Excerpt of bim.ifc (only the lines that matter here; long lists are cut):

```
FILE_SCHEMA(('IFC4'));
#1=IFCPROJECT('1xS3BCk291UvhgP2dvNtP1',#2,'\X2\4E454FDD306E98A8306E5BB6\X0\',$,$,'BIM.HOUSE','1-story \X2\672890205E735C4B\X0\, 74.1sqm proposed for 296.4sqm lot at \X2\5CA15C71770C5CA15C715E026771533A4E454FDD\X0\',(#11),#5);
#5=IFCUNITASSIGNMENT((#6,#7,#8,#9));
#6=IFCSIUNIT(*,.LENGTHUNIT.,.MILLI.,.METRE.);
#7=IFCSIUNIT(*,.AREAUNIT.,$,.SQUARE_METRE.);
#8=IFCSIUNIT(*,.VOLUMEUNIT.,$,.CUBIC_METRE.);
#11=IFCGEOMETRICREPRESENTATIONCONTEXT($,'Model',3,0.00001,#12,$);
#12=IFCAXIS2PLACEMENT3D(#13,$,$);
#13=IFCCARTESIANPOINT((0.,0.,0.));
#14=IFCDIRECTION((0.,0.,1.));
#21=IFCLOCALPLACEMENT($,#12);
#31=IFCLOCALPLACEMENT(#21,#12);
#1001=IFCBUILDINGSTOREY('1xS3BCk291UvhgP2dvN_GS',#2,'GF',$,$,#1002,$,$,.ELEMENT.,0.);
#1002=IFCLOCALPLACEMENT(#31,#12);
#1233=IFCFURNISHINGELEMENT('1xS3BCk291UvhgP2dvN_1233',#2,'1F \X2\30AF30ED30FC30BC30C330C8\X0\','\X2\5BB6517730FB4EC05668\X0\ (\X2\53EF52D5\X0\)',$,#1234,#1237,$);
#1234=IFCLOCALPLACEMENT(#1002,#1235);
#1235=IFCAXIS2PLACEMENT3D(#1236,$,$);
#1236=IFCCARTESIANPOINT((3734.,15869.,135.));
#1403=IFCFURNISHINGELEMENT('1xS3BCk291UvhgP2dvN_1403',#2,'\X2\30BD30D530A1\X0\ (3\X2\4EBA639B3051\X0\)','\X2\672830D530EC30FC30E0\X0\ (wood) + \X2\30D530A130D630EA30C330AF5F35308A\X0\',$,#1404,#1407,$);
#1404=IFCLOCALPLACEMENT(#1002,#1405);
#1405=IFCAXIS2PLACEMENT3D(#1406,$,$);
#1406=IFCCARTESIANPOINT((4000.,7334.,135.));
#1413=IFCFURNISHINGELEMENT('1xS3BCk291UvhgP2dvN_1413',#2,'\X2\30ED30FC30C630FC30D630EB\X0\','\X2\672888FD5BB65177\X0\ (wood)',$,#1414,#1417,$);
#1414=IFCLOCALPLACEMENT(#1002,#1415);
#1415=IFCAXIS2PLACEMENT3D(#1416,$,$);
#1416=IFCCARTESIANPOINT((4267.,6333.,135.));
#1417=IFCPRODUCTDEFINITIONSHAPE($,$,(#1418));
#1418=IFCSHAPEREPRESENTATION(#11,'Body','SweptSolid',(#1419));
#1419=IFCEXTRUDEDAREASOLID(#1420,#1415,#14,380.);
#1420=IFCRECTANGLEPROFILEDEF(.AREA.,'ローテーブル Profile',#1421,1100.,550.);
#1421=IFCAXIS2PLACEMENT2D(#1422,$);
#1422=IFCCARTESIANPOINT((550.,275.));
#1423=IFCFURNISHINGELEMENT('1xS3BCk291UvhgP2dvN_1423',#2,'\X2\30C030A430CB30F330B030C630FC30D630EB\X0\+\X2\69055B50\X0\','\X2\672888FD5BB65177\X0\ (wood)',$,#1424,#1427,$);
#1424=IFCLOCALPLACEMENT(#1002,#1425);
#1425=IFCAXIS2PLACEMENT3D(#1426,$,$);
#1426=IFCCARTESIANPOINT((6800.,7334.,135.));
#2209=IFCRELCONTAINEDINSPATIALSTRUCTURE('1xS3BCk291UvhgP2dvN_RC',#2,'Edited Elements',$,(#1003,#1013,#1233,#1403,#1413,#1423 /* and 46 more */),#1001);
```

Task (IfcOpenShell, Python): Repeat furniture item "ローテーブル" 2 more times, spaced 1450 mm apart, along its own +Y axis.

```python
import ifcopenshell
import ifcopenshell.api.geometry
import ifcopenshell.api.root
import ifcopenshell.util.element
import ifcopenshell.util.placement
import ifcopenshell.util.unit

model = ifcopenshell.open("bim.ifc")
unit_scale = ifcopenshell.util.unit.calculate_unit_scale(model)


def reuse_history(source, copy):
    """copy_class also copies each property set's owner history, people and application; keep the originals."""
    for rel in copy.IsDefinedBy:
        if rel.is_a("IfcRelDefinesByProperties") and (history := rel.RelatingPropertyDefinition.OwnerHistory):
            rel.RelatingPropertyDefinition.OwnerHistory = source.OwnerHistory
            ifcopenshell.util.element.remove_deep2(model, history)


source = model.by_id(1413)
base = ifcopenshell.util.placement.get_local_placement(source.ObjectPlacement)
step = base[:3, 1] * 1.45 / unit_scale

for i in range(1, 3):
    copy = ifcopenshell.api.root.copy_class(model, product=source)
    copy.Representation = ifcopenshell.util.element.copy_deep(
        model, source.Representation, exclude=["IfcGeometricRepresentationContext", "IfcRepresentationMap"]
    )
    reuse_history(source, copy)
    matrix = base.copy()
    matrix[:3, 3] += i * step
    print("added at", matrix[:3, 3].round(3) + 0.0)
    ifcopenshell.api.geometry.edit_object_placement(model, product=copy, matrix=matrix, is_si=False)

model.write("bim-out.ifc")
```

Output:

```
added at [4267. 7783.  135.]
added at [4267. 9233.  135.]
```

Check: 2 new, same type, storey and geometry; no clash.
